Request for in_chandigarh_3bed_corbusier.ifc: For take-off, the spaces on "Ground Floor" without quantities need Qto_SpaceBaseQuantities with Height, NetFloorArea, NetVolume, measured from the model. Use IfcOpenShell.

First a look at what the model holds.

```python
import ifcopenshell
import ifcopenshell.util.element
import ifcopenshell.util.unit

model = ifcopenshell.open("in_chandigarh_3bed_corbusier.ifc")
print(model.schema)
for unit_type in ("LENGTHUNIT", "AREAUNIT", "VOLUMEUNIT"):
    print(unit_type, ifcopenshell.util.unit.calculate_unit_scale(model, unit_type))
storey = next(s for s in model.by_type("IfcBuildingStorey") if s.Name == "Ground Floor")
spaces = [e for e in ifcopenshell.util.element.get_decomposition(storey) if e.is_a("IfcSpace")]
for e in sorted(spaces, key=lambda e: e.id()):
    print(e.id(), e.is_a(), e.Name, list(ifcopenshell.util.element.get_psets(e, qtos_only=True)), sep=" | ")
```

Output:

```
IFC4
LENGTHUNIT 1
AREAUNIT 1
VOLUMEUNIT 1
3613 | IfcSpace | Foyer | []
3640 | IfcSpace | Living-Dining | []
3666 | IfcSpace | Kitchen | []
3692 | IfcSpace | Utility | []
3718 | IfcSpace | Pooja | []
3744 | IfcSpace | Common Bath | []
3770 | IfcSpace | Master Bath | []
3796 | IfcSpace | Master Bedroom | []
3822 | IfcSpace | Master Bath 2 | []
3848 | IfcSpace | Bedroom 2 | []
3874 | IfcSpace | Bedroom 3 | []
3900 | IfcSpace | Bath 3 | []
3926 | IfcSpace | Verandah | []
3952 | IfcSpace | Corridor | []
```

```python
import ifcopenshell
import ifcopenshell.api.pset
import ifcopenshell.geom
import ifcopenshell.util.element
import ifcopenshell.util.shape
import ifcopenshell.util.unit

model = ifcopenshell.open("in_chandigarh_3bed_corbusier.ifc")
unit_scale = ifcopenshell.util.unit.calculate_unit_scale(model)
area_scale = ifcopenshell.util.unit.calculate_unit_scale(model, "AREAUNIT")
volume_scale = ifcopenshell.util.unit.calculate_unit_scale(model, "VOLUMEUNIT")
settings = ifcopenshell.geom.settings()

storey = next(s for s in model.by_type("IfcBuildingStorey") if s.Name == "Ground Floor")
spaces = [e for e in ifcopenshell.util.element.get_decomposition(storey) if e.is_a("IfcSpace")]

for e in sorted(spaces, key=lambda e: e.id()):
    if ifcopenshell.util.element.get_psets(e, qtos_only=True, should_inherit=False):
        continue
    # Geometry comes back in metres, in the element's own axes.
    shape = ifcopenshell.geom.create_shape(settings, e)
    values = {
        "Height": ifcopenshell.util.shape.get_z(shape.geometry) / unit_scale,
        "NetFloorArea": ifcopenshell.util.shape.get_footprint_area(shape.geometry) / area_scale,
        "NetVolume": ifcopenshell.util.shape.get_volume(shape.geometry) / volume_scale,
    }
    qto = ifcopenshell.api.pset.add_qto(model, product=e, name="Qto_SpaceBaseQuantities")
    ifcopenshell.api.pset.edit_qto(model, qto=qto, properties=values)
    print(e.id(), {k: round(v, 3) for k, v in values.items()})

model.write("in_chandigarh_3bed_corbusier_edited.ifc")
```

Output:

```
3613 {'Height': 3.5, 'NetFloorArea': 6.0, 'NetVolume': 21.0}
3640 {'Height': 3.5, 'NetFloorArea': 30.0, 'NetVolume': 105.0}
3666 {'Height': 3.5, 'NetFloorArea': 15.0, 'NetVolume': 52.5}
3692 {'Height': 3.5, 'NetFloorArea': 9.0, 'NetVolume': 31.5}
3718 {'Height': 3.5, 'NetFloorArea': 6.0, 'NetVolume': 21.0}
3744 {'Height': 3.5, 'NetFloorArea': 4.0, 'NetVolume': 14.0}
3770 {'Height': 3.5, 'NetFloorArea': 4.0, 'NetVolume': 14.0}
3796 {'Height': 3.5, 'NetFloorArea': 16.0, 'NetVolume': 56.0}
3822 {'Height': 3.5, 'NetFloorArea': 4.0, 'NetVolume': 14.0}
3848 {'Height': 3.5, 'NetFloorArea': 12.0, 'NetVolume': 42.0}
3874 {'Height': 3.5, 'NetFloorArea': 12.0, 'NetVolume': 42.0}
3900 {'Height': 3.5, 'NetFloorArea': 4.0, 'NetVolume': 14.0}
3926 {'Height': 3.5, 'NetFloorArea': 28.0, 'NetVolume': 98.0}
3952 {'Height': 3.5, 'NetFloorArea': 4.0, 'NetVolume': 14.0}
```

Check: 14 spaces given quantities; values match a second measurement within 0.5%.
